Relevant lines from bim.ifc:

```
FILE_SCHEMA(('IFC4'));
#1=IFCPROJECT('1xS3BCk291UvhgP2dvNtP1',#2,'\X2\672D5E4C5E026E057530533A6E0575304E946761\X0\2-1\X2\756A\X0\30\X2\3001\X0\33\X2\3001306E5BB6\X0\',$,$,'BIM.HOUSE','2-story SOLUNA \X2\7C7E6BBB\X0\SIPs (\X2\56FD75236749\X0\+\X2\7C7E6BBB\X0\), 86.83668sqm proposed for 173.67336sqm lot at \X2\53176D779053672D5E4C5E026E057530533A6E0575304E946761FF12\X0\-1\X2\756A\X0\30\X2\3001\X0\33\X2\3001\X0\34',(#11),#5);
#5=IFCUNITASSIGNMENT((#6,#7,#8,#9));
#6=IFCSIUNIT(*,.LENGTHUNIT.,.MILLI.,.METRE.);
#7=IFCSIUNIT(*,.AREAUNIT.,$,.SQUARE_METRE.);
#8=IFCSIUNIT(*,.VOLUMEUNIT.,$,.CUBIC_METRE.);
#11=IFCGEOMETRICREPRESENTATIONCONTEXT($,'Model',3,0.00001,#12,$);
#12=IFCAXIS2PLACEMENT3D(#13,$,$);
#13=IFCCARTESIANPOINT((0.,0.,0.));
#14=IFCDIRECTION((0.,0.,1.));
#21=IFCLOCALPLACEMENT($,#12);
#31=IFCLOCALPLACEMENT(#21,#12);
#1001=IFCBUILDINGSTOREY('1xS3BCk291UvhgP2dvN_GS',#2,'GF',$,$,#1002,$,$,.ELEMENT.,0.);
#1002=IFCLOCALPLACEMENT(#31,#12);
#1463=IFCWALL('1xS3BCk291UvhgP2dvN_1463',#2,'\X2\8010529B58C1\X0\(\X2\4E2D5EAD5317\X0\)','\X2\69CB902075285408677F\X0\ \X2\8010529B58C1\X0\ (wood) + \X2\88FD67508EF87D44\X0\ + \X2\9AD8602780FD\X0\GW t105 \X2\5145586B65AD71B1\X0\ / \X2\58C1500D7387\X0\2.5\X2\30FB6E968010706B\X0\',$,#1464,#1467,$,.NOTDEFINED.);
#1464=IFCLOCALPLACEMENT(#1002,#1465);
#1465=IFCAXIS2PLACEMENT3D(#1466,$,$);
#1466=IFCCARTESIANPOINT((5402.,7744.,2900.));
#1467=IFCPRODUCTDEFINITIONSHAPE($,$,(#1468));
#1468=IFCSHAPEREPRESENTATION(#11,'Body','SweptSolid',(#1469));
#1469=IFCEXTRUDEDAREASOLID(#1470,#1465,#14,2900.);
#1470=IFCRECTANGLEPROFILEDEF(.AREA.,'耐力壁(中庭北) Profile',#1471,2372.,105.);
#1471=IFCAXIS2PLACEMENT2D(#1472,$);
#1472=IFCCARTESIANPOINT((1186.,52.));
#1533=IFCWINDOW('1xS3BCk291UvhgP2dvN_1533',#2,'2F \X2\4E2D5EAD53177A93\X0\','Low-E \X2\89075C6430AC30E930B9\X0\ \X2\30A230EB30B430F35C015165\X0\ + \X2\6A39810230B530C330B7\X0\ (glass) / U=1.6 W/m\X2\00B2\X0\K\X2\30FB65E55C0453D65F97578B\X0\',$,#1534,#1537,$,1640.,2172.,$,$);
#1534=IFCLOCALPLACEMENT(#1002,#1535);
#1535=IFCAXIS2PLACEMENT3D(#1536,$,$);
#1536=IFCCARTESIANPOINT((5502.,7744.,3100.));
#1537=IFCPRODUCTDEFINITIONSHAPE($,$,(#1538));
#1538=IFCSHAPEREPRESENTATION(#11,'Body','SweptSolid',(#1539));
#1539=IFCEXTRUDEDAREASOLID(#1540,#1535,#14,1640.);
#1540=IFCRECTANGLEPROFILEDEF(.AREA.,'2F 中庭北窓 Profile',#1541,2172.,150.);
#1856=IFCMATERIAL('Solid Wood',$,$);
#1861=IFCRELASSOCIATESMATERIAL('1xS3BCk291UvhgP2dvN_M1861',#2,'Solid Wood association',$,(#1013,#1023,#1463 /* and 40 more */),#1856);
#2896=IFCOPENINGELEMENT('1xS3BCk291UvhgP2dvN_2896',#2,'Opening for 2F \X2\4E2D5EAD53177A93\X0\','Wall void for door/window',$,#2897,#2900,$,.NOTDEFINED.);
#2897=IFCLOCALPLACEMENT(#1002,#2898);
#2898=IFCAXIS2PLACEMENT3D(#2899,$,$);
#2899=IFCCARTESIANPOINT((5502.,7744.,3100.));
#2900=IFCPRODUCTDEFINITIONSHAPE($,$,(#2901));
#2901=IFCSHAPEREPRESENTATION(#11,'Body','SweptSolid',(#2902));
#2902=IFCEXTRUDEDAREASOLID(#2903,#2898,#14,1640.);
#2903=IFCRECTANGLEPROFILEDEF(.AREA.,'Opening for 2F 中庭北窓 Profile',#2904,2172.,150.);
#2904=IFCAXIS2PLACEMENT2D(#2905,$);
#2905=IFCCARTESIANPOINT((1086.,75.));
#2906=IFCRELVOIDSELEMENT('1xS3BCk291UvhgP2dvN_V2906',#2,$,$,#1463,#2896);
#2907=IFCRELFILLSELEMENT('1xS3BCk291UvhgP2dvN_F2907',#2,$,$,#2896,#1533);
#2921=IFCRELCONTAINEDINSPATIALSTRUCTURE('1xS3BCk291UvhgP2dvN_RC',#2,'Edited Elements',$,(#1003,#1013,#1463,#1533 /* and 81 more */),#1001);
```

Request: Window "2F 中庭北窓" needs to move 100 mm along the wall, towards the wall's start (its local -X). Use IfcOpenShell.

```python
import ifcopenshell
import ifcopenshell.api.geometry
import ifcopenshell.util.placement
import ifcopenshell.util.unit

model = ifcopenshell.open("bim.ifc")
unit_scale = ifcopenshell.util.unit.calculate_unit_scale(model)

window = model.by_id(1533)
opening = window.FillsVoids[0].RelatingOpeningElement
wall = opening.VoidsElements[0].RelatingBuildingElement

wall_matrix = ifcopenshell.util.placement.get_local_placement(wall.ObjectPlacement)
shift = wall_matrix[:3, 0] * -0.1 / unit_scale
before = ifcopenshell.util.placement.get_local_placement(window.ObjectPlacement)[:3, 3].copy()

# The window is not placed relative to its opening, so move both.
for product in (opening, window):
    matrix = ifcopenshell.util.placement.get_local_placement(product.ObjectPlacement)
    matrix[:3, 3] += shift
    ifcopenshell.api.geometry.edit_object_placement(model, product=product, matrix=matrix, is_si=False)

after = ifcopenshell.util.placement.get_local_placement(window.ObjectPlacement)[:3, 3]
print("window moved by", (after - before).round(3) + 0.0)

model.write("bim_v2.ifc")
```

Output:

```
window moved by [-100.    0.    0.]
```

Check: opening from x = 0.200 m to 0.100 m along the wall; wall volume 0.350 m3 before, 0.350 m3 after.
